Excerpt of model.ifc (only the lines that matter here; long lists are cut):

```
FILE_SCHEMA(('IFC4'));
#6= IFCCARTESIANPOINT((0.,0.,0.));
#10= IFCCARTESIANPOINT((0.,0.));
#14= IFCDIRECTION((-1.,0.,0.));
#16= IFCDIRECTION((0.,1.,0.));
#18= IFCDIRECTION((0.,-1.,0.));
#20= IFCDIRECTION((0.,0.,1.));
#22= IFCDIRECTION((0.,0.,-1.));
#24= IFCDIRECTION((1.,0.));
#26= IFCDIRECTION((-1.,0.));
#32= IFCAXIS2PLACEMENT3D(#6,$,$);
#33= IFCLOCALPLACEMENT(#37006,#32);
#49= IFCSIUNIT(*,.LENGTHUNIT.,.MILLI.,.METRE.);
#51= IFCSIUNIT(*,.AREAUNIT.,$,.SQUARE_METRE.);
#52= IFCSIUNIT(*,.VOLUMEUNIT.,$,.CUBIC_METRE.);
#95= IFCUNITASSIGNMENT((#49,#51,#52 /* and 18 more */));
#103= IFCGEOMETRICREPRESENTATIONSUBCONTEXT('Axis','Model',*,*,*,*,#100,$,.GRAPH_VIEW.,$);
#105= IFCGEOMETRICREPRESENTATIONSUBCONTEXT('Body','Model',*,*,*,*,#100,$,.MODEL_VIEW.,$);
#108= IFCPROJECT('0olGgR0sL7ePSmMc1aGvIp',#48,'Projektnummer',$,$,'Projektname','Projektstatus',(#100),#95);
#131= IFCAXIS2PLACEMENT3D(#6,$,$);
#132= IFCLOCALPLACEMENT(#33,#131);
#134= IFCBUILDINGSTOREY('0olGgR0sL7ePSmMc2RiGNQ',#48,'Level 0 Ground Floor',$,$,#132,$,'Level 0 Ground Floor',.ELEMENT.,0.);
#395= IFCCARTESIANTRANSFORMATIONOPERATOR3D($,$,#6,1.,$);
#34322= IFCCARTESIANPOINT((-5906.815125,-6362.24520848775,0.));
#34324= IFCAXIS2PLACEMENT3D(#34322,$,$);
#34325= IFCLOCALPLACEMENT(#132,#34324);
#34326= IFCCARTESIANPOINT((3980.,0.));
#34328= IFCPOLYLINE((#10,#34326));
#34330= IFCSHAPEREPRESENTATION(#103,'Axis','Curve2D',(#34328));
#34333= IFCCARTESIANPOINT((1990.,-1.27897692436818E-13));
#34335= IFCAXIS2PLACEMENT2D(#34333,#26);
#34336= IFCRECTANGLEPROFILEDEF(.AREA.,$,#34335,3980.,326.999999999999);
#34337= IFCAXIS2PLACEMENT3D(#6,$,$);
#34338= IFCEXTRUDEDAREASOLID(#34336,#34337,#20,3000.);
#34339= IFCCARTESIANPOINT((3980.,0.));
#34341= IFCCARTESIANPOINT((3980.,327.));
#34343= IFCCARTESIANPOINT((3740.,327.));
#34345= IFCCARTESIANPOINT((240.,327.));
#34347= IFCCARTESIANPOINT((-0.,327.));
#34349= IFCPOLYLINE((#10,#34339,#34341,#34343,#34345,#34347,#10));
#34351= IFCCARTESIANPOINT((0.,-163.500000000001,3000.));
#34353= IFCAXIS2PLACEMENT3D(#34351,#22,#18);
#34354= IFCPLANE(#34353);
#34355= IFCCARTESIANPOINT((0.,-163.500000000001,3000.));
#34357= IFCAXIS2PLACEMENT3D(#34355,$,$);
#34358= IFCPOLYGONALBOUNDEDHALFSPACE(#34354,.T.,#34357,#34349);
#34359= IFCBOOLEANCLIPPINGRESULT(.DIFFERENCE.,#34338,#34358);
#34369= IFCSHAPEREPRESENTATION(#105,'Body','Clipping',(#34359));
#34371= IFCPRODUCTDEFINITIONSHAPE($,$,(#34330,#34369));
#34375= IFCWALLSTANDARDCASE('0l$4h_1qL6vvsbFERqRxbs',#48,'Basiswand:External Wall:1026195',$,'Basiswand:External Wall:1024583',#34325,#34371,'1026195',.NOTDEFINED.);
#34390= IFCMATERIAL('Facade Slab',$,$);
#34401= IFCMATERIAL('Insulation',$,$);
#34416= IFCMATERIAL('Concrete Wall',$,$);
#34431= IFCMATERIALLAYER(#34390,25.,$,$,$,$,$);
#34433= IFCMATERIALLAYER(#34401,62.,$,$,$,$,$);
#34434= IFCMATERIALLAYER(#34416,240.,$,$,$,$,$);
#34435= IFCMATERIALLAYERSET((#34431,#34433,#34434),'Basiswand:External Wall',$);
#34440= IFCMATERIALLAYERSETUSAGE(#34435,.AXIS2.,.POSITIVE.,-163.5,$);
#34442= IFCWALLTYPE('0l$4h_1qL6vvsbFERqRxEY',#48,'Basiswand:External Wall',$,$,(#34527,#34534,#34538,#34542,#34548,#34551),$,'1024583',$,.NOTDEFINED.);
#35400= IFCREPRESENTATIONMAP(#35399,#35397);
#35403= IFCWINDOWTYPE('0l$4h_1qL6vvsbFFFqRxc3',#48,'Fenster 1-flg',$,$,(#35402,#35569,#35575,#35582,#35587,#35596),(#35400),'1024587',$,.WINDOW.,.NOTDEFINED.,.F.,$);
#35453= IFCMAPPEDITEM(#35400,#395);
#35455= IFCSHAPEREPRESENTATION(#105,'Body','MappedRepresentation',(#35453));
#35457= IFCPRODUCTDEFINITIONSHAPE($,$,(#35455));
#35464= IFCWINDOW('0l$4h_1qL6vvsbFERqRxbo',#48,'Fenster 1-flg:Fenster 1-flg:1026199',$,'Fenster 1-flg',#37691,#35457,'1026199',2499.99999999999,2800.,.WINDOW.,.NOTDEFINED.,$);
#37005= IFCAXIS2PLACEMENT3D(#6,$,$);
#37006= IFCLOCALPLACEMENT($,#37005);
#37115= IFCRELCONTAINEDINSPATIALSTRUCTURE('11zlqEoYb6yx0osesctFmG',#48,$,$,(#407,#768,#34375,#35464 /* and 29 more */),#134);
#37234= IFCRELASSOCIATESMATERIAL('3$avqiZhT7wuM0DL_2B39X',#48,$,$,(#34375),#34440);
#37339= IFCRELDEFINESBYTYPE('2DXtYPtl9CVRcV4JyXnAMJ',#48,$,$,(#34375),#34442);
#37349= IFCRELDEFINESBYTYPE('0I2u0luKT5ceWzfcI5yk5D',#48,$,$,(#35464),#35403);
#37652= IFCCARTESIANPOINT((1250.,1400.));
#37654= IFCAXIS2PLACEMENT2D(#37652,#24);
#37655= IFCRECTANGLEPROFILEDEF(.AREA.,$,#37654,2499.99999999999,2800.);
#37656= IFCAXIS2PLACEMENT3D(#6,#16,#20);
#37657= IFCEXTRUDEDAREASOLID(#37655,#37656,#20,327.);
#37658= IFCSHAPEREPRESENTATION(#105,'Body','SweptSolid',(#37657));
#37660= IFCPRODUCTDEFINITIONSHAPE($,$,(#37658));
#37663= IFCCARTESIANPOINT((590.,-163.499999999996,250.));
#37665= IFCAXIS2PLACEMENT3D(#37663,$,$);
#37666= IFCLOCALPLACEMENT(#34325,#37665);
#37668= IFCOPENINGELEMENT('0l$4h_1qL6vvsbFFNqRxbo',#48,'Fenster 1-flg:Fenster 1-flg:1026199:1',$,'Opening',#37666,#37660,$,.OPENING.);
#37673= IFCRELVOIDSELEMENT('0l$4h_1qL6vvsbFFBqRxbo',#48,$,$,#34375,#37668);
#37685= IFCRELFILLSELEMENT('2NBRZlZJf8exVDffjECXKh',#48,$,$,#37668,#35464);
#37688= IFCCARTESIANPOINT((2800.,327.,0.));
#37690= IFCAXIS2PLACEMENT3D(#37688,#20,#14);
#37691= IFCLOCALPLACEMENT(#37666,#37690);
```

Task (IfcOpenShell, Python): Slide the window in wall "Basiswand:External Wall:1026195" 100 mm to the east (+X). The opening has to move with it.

```python
import ifcopenshell
import ifcopenshell.api.geometry
import ifcopenshell.util.placement
import ifcopenshell.util.unit

model = ifcopenshell.open("model.ifc")
unit_scale = ifcopenshell.util.unit.calculate_unit_scale(model)

window = model.by_id(35464)
opening = window.FillsVoids[0].RelatingOpeningElement
wall = opening.VoidsElements[0].RelatingBuildingElement

wall_matrix = ifcopenshell.util.placement.get_local_placement(wall.ObjectPlacement)
shift = wall_matrix[:3, 0] * 0.1 / unit_scale
before = ifcopenshell.util.placement.get_local_placement(window.ObjectPlacement)[:3, 3].copy()

# The window is placed relative to its opening, so it follows when the opening moves.
matrix = ifcopenshell.util.placement.get_local_placement(opening.ObjectPlacement)
matrix[:3, 3] += shift
ifcopenshell.api.geometry.edit_object_placement(
    model, product=opening, matrix=matrix, is_si=False, should_transform_children=True
)

after = ifcopenshell.util.placement.get_local_placement(window.ObjectPlacement)[:3, 3]
print("window moved by", (after - before).round(3) + 0.0)

model.write("model_updated.ifc")
```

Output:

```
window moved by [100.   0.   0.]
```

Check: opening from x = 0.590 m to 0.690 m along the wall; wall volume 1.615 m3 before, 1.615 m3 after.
